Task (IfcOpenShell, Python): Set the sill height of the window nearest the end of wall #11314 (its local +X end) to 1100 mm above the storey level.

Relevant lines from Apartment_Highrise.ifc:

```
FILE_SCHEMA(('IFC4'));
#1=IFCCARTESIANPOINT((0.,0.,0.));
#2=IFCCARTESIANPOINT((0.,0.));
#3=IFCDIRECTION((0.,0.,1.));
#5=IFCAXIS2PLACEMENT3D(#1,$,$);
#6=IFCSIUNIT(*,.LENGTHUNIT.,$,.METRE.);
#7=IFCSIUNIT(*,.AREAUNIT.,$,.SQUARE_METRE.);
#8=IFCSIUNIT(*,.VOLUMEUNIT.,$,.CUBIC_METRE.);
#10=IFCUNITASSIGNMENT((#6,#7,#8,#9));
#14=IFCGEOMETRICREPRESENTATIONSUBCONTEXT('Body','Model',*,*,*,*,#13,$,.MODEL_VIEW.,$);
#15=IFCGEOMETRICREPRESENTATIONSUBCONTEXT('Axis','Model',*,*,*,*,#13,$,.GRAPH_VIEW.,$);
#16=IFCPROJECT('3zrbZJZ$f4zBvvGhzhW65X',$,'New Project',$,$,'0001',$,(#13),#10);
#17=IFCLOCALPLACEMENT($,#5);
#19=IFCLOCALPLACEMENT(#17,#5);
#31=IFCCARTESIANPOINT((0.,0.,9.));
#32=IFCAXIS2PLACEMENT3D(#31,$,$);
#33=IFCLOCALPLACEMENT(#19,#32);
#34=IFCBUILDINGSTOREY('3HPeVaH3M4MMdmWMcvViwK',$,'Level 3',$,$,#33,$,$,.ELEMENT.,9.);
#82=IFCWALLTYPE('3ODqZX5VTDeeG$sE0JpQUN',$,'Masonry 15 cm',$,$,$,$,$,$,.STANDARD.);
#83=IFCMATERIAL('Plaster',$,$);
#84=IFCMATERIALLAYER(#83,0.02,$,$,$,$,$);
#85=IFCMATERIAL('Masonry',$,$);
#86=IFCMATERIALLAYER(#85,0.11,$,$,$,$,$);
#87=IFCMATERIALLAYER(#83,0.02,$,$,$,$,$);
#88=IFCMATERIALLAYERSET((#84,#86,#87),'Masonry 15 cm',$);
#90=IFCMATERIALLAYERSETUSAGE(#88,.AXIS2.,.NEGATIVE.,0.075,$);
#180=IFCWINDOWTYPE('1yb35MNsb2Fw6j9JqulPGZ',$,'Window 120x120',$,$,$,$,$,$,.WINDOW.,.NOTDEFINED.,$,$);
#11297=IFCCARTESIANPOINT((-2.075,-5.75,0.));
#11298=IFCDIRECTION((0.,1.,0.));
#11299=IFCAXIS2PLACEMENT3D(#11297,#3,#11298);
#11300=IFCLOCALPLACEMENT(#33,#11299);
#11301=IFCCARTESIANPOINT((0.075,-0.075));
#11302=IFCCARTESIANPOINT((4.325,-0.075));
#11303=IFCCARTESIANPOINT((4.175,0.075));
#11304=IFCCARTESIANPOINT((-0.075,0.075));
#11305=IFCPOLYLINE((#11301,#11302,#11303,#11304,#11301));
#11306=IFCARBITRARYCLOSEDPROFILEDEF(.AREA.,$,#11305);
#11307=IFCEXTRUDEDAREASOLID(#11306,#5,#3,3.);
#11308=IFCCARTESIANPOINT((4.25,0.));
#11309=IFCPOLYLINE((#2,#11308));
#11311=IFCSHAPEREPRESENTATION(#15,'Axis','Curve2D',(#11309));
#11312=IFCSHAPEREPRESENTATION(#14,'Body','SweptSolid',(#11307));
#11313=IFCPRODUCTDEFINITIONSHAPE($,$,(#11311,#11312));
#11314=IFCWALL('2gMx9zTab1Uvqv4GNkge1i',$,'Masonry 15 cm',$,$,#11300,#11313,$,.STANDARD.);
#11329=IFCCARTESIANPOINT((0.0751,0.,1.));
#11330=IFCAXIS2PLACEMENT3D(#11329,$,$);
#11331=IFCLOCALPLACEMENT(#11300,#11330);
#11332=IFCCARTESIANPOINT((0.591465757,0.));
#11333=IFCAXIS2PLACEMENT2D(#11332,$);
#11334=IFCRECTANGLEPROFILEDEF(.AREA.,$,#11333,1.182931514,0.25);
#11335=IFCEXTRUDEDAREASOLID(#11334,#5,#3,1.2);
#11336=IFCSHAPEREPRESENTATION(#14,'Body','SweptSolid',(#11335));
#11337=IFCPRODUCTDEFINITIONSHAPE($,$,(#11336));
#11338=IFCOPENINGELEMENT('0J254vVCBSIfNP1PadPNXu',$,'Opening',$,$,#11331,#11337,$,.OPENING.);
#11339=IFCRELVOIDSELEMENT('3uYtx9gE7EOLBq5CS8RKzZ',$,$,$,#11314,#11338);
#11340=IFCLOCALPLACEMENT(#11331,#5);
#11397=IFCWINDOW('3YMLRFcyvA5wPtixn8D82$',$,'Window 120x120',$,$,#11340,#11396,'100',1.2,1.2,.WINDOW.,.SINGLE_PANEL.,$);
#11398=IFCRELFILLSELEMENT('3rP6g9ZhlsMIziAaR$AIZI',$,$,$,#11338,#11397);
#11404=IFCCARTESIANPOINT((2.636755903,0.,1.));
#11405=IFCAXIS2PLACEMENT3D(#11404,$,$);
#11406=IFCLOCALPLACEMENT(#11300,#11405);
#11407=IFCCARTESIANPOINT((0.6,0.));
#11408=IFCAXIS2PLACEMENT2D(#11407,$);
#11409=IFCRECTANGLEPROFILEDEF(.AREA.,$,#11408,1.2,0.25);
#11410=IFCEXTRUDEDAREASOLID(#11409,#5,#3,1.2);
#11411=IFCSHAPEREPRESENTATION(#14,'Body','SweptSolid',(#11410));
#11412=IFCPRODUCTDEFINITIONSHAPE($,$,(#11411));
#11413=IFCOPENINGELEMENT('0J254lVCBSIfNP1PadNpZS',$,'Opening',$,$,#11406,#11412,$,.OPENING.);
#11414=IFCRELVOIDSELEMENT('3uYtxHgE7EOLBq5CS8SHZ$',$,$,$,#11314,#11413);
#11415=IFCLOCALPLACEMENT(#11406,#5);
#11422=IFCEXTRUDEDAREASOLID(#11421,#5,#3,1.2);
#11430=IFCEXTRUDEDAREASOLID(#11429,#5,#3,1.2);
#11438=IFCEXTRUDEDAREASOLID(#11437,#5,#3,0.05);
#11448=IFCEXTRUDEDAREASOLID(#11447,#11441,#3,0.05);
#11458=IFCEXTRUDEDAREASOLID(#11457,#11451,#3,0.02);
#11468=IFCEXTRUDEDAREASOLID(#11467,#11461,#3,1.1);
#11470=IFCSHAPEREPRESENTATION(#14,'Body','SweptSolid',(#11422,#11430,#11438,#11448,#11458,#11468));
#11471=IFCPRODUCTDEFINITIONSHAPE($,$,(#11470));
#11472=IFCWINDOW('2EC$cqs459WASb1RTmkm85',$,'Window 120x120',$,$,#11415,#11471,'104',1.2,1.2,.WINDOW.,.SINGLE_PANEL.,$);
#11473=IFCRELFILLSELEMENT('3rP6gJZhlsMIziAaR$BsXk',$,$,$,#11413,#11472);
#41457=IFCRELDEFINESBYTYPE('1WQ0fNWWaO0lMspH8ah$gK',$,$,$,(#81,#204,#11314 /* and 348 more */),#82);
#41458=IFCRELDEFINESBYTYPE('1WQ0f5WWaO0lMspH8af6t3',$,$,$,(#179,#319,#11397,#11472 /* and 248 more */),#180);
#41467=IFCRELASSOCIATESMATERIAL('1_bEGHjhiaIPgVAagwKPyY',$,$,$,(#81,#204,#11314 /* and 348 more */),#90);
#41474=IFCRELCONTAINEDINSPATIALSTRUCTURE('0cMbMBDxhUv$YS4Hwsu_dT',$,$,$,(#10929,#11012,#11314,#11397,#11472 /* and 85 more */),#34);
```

```python
import numpy as np
import ifcopenshell
import ifcopenshell.api.geometry
import ifcopenshell.geom
import ifcopenshell.util.element
import ifcopenshell.util.placement
import ifcopenshell.util.shape
import ifcopenshell.util.unit

model = ifcopenshell.open("Apartment_Highrise.ifc")
unit_scale = ifcopenshell.util.unit.calculate_unit_scale(model)

window = model.by_guid("2EC$cqs459WASb1RTmkm85")
opening = window.FillsVoids[0].RelatingOpeningElement
storey = ifcopenshell.util.element.get_container(window, ifc_class="IfcBuildingStorey")
level = ifcopenshell.util.placement.get_local_placement(storey.ObjectPlacement)[2, 3]

# The opening's origin need not be at the sill, so measure its lowest point.
shape = ifcopenshell.geom.create_shape(ifcopenshell.geom.settings(), opening)
bottom = ifcopenshell.util.shape.get_shape_bottom_elevation(shape, shape.geometry) / unit_scale
dz = level + 1.1 / unit_scale - bottom

shift = np.array([0.0, 0.0, dz])
# The window is placed relative to its opening, so it follows when the opening moves.
matrix = ifcopenshell.util.placement.get_local_placement(opening.ObjectPlacement)
matrix[:3, 3] += shift
ifcopenshell.api.geometry.edit_object_placement(
    model, product=opening, matrix=matrix, is_si=False, should_transform_children=True
)

print(f"moved by {dz * unit_scale:+.3f} m")

model.write("Apartment_Highrise_edited.ifc")
```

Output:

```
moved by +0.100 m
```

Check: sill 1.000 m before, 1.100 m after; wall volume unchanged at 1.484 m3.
